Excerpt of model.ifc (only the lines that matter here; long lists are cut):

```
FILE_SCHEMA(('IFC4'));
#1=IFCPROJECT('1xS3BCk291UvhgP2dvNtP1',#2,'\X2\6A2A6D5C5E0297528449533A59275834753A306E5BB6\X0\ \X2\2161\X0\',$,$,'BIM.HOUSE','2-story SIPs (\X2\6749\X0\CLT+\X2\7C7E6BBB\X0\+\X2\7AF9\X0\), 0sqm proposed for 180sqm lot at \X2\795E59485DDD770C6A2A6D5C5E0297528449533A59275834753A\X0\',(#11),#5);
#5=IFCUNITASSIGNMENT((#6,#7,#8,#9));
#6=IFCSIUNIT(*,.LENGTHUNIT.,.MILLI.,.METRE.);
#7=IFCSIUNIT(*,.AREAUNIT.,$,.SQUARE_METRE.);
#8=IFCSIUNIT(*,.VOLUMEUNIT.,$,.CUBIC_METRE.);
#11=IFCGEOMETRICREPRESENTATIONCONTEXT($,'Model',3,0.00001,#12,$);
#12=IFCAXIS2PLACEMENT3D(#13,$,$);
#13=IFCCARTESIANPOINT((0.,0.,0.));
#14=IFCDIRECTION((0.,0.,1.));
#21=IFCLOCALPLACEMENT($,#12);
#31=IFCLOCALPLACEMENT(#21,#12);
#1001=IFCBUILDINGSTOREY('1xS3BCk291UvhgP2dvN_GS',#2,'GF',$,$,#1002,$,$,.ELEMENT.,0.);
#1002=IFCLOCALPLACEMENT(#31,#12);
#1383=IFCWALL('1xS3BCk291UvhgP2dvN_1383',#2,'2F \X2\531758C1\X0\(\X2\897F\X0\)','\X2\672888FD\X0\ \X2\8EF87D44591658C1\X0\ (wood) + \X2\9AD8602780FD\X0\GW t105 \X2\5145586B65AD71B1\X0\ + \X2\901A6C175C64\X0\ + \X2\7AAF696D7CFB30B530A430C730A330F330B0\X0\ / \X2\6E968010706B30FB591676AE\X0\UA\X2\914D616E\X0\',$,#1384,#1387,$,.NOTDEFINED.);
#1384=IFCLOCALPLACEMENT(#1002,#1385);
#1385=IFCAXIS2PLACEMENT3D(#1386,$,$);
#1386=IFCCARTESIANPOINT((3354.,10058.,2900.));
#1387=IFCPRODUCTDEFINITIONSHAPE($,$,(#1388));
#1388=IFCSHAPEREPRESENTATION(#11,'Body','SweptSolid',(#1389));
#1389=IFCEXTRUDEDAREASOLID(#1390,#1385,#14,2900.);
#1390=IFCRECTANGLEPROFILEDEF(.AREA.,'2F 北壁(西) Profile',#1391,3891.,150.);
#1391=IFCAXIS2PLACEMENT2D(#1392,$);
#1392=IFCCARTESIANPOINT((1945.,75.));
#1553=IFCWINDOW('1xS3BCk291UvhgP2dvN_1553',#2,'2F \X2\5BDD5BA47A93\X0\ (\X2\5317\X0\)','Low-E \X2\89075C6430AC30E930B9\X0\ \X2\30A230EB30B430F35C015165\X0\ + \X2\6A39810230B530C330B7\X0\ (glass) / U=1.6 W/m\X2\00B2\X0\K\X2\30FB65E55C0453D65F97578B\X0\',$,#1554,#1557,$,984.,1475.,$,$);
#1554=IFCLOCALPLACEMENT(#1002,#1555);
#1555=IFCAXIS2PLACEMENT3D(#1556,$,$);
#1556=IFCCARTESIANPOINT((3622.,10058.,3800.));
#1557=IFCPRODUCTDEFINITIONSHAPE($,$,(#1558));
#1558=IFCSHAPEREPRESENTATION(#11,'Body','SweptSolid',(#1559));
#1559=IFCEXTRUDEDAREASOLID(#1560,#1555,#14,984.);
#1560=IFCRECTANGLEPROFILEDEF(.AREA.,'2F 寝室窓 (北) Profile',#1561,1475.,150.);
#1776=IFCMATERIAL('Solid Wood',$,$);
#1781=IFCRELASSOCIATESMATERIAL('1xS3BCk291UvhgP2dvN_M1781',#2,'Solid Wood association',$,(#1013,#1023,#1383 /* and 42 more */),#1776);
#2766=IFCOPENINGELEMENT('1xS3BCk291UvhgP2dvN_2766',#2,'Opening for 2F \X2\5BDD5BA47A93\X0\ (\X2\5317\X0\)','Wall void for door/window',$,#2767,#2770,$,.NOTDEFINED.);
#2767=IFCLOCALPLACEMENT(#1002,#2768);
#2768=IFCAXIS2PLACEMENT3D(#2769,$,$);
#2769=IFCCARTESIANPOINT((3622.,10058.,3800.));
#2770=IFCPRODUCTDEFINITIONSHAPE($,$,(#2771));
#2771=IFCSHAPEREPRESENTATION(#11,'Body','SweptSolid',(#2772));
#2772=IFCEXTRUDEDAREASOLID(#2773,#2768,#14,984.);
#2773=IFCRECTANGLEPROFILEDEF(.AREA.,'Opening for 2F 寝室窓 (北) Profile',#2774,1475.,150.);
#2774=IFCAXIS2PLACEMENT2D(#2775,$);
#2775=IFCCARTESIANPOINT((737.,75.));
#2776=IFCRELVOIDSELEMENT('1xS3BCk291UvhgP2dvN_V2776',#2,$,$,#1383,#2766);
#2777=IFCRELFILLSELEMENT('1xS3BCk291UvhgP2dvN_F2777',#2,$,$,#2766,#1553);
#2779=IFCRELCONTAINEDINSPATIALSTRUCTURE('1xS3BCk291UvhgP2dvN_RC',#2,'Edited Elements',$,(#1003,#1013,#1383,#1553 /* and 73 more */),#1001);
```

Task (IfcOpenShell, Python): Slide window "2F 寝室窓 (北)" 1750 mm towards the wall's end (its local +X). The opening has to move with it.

```python
import ifcopenshell
import ifcopenshell.api.geometry
import ifcopenshell.util.placement
import ifcopenshell.util.unit

model = ifcopenshell.open("model.ifc")
unit_scale = ifcopenshell.util.unit.calculate_unit_scale(model)

window = model.by_guid("1xS3BCk291UvhgP2dvN_1553")
opening = window.FillsVoids[0].RelatingOpeningElement
wall = opening.VoidsElements[0].RelatingBuildingElement

wall_matrix = ifcopenshell.util.placement.get_local_placement(wall.ObjectPlacement)
shift = wall_matrix[:3, 0] * 1.75 / unit_scale
before = ifcopenshell.util.placement.get_local_placement(window.ObjectPlacement)[:3, 3].copy()

# The window is not placed relative to its opening, so move both.
for product in (opening, window):
    matrix = ifcopenshell.util.placement.get_local_placement(product.ObjectPlacement)
    matrix[:3, 3] += shift
    ifcopenshell.api.geometry.edit_object_placement(model, product=product, matrix=matrix, is_si=False)

after = ifcopenshell.util.placement.get_local_placement(window.ObjectPlacement)[:3, 3]
print("window moved by", (after - before).round(3) + 0.0)

model.write("model_edited.ifc")
```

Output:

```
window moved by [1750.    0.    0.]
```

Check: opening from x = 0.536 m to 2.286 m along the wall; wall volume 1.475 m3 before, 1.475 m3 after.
